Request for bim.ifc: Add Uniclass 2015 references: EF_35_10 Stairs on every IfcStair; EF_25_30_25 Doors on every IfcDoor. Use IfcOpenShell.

First a look at what the model holds.

```python
import ifcopenshell

model = ifcopenshell.open("bim.ifc")
print(model.schema)
print("classifications:", [c.Name for c in model.by_type("IfcClassification")])
for ifc_class in ("IfcDoor", "IfcRoof", "IfcStair", "IfcWall", "IfcWindow"):
    print(ifc_class, len(model.by_type(ifc_class)))
```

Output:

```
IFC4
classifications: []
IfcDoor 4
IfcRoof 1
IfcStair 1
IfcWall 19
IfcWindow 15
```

```python
import ifcopenshell
import ifcopenshell.api.classification

model = ifcopenshell.open("bim.ifc")

system = ifcopenshell.api.classification.add_classification(model, classification="Uniclass 2015")

codes = {
    "IfcStair": ("EF_35_10", "Stairs"),
    "IfcDoor": ("EF_25_30_25", "Doors"),
}
for ifc_class, (code, name) in codes.items():
    products = model.by_type(ifc_class)
    ifcopenshell.api.classification.add_reference(
        model, products=products, classification=system, identification=code, name=name
    )
    print(code, len(products))

model.write("bim_updated.ifc")
```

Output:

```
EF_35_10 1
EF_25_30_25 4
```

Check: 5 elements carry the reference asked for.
